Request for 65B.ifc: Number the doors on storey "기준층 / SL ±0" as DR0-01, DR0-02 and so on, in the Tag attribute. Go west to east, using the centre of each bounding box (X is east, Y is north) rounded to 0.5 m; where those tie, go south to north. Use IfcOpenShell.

First a look at what the model holds.

```python
import ifcopenshell
import ifcopenshell.util.element
import ifcopenshell.util.placement

model = ifcopenshell.open("65B.ifc")
print(model.schema)
storey = next(s for s in model.by_type("IfcBuildingStorey") if s.Name == "기준층 / SL ±0")
doors = [e for e in ifcopenshell.util.element.get_decomposition(storey) if e.is_a("IfcDoor")]
for e in sorted(doors, key=lambda e: e.id()):
    origin = ifcopenshell.util.placement.get_local_placement(e.ObjectPlacement)[:3, 3]
    print(e.id(), e.Tag, e.Name, origin.round(2) + 0.0, sep=" | ")
```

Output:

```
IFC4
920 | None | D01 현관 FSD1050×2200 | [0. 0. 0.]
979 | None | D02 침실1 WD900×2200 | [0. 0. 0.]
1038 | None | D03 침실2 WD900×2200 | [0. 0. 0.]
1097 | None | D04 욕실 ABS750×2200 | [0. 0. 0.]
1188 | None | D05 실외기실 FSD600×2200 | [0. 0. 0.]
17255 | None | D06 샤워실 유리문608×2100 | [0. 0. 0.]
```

```python
import ifcopenshell
import ifcopenshell.geom
import ifcopenshell.util.element
import ifcopenshell.util.shape

model = ifcopenshell.open("65B.ifc")
settings = ifcopenshell.geom.settings()
settings.set("use-world-coords", True)


def centre(element):
    shape = ifcopenshell.geom.create_shape(settings, element)
    return ifcopenshell.util.shape.get_bbox_centroid(shape.geometry)


storey = next(s for s in model.by_type("IfcBuildingStorey") if s.Name == "기준층 / SL ±0")
doors = [e for e in ifcopenshell.util.element.get_decomposition(storey) if e.is_a("IfcDoor")]

# Insertion points can sit at a corner or the storey origin, so sort by the geometry (in metres).
centres = {e: centre(e) for e in doors}
doors.sort(key=lambda e: (round(centres[e][0] / 0.5), centres[e][1]))

for i, e in enumerate(doors, start=1):
    number = f"DR0-{i:02d}"
    e.Tag = number
    print(e.id(), number)

model.write("65B-out.ifc")
```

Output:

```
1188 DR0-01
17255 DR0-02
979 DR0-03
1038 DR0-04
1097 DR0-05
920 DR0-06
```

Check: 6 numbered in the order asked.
